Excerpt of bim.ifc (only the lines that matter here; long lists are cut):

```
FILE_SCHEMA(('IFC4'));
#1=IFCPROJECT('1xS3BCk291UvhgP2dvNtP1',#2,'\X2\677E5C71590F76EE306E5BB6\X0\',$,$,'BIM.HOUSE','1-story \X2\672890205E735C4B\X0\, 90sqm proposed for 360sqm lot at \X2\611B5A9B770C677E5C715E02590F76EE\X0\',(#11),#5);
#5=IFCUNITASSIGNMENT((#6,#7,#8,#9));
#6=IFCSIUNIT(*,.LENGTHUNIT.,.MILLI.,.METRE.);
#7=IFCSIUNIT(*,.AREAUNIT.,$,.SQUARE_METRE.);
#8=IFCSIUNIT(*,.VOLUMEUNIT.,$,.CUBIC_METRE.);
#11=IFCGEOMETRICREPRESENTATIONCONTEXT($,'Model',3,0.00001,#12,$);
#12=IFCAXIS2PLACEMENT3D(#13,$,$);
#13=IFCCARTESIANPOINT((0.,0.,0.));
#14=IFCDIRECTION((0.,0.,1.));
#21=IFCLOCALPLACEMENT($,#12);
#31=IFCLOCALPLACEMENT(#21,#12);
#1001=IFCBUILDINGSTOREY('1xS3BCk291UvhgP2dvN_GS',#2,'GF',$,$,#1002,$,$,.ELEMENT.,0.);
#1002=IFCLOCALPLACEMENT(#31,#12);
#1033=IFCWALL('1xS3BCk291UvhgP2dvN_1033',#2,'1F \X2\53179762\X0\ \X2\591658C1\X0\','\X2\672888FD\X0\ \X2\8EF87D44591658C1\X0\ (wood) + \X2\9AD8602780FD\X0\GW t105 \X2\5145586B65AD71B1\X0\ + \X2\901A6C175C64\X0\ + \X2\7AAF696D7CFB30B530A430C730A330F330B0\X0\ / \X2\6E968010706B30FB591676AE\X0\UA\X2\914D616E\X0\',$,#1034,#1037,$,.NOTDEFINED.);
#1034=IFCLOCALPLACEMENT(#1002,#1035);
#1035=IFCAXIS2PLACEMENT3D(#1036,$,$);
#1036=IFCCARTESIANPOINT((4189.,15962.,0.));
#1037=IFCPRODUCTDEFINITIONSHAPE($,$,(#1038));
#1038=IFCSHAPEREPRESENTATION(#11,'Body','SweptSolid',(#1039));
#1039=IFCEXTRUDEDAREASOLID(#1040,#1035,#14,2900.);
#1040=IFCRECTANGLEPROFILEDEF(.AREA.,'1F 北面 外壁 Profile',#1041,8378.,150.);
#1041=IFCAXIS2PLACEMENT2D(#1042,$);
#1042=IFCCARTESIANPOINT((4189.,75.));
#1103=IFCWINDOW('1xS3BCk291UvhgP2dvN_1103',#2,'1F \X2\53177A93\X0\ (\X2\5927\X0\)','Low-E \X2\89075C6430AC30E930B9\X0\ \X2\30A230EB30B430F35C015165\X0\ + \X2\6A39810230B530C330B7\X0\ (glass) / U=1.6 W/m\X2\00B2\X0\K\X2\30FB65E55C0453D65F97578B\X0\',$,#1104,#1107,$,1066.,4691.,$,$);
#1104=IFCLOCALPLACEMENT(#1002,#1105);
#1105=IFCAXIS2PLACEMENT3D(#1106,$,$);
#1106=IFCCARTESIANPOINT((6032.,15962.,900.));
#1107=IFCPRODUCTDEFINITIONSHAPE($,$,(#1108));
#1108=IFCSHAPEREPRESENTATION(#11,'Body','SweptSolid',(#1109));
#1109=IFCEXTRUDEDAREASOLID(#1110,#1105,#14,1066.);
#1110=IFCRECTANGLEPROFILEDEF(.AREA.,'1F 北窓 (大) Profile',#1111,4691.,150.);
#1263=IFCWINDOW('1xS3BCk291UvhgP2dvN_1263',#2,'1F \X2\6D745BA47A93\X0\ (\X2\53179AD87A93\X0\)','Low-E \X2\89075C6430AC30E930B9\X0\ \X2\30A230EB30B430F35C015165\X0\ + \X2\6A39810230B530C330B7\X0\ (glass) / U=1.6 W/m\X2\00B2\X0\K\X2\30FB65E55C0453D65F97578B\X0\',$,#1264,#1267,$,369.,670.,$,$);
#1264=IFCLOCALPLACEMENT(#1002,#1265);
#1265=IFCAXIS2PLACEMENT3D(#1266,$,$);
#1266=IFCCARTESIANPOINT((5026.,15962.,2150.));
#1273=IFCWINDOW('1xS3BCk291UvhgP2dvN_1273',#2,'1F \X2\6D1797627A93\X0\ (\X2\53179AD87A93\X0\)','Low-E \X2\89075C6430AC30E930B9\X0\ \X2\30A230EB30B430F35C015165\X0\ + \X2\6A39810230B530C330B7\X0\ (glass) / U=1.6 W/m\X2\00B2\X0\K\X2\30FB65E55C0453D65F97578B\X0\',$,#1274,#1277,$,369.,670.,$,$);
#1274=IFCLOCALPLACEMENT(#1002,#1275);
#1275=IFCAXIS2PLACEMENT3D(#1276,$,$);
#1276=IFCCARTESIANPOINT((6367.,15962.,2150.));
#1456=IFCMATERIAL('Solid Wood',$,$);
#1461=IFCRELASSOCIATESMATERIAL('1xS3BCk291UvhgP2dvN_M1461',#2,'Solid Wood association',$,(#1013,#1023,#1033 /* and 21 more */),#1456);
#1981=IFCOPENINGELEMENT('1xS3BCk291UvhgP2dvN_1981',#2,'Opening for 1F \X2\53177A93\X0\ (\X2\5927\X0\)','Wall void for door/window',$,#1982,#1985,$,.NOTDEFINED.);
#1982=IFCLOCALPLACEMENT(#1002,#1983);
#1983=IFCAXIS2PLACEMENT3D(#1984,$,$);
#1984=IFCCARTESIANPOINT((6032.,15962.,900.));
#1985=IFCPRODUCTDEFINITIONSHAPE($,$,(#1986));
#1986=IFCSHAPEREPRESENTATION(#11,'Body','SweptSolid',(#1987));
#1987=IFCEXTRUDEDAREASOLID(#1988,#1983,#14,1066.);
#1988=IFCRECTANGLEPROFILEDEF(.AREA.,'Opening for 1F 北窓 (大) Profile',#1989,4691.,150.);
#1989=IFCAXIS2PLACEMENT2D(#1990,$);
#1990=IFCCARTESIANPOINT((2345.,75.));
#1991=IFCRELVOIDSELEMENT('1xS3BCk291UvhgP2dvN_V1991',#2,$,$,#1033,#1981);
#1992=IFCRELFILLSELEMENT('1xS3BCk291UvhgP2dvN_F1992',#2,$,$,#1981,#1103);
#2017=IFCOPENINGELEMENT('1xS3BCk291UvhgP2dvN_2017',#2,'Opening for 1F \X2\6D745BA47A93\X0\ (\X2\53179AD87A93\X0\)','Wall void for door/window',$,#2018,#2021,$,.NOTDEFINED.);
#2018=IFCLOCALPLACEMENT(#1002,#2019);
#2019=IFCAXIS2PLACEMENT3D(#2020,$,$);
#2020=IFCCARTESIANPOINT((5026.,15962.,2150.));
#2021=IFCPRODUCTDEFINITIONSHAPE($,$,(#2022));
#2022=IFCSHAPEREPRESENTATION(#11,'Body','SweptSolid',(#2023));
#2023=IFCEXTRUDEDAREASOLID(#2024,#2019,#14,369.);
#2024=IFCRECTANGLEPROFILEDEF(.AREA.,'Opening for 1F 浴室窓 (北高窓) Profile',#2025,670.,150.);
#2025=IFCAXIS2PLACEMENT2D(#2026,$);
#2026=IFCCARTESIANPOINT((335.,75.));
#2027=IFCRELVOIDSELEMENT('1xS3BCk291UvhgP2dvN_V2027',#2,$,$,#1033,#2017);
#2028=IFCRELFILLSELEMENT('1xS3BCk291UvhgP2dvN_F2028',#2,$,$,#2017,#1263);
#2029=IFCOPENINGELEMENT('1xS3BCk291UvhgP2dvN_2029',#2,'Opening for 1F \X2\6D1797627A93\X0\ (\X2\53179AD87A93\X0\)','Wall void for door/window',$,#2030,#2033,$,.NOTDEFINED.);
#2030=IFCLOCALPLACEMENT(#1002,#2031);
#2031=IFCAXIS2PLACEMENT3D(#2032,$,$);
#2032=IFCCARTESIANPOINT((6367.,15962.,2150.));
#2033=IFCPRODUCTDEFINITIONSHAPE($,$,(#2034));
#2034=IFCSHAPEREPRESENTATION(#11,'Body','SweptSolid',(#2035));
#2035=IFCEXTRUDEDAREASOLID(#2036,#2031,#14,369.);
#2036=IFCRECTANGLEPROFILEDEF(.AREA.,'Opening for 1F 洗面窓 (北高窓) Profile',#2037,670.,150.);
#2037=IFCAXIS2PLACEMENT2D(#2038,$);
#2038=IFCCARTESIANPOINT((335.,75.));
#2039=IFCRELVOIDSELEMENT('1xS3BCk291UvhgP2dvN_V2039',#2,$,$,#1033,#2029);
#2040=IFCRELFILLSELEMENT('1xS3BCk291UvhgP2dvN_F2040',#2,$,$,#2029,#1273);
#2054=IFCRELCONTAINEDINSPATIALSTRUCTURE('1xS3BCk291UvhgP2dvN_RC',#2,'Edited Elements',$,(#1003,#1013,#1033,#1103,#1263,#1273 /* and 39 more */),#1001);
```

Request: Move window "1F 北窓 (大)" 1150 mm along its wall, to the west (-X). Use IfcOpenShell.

```python
import ifcopenshell
import ifcopenshell.api.geometry
import ifcopenshell.util.placement

model = ifcopenshell.open("bim.ifc")

window = model.by_guid("1xS3BCk291UvhgP2dvN_1103")
opening = window.FillsVoids[0].RelatingOpeningElement
wall = opening.VoidsElements[0].RelatingBuildingElement

wall_matrix = ifcopenshell.util.placement.get_local_placement(wall.ObjectPlacement)
shift = wall_matrix[:3, 0] * -1150.0
before = ifcopenshell.util.placement.get_local_placement(window.ObjectPlacement)[:3, 3].copy()

# The window is not placed relative to its opening, so move both.
for product in (opening, window):
    matrix = ifcopenshell.util.placement.get_local_placement(product.ObjectPlacement)
    matrix[:3, 3] += shift
    ifcopenshell.api.geometry.edit_object_placement(model, product=product, matrix=matrix, is_si=False)

after = ifcopenshell.util.placement.get_local_placement(window.ObjectPlacement)[:3, 3]
print("window moved by", (after - before).round(3) + 0.0)

model.write("bim-out.ifc")
```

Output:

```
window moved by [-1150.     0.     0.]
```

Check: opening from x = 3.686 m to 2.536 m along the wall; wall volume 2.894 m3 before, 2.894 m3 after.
